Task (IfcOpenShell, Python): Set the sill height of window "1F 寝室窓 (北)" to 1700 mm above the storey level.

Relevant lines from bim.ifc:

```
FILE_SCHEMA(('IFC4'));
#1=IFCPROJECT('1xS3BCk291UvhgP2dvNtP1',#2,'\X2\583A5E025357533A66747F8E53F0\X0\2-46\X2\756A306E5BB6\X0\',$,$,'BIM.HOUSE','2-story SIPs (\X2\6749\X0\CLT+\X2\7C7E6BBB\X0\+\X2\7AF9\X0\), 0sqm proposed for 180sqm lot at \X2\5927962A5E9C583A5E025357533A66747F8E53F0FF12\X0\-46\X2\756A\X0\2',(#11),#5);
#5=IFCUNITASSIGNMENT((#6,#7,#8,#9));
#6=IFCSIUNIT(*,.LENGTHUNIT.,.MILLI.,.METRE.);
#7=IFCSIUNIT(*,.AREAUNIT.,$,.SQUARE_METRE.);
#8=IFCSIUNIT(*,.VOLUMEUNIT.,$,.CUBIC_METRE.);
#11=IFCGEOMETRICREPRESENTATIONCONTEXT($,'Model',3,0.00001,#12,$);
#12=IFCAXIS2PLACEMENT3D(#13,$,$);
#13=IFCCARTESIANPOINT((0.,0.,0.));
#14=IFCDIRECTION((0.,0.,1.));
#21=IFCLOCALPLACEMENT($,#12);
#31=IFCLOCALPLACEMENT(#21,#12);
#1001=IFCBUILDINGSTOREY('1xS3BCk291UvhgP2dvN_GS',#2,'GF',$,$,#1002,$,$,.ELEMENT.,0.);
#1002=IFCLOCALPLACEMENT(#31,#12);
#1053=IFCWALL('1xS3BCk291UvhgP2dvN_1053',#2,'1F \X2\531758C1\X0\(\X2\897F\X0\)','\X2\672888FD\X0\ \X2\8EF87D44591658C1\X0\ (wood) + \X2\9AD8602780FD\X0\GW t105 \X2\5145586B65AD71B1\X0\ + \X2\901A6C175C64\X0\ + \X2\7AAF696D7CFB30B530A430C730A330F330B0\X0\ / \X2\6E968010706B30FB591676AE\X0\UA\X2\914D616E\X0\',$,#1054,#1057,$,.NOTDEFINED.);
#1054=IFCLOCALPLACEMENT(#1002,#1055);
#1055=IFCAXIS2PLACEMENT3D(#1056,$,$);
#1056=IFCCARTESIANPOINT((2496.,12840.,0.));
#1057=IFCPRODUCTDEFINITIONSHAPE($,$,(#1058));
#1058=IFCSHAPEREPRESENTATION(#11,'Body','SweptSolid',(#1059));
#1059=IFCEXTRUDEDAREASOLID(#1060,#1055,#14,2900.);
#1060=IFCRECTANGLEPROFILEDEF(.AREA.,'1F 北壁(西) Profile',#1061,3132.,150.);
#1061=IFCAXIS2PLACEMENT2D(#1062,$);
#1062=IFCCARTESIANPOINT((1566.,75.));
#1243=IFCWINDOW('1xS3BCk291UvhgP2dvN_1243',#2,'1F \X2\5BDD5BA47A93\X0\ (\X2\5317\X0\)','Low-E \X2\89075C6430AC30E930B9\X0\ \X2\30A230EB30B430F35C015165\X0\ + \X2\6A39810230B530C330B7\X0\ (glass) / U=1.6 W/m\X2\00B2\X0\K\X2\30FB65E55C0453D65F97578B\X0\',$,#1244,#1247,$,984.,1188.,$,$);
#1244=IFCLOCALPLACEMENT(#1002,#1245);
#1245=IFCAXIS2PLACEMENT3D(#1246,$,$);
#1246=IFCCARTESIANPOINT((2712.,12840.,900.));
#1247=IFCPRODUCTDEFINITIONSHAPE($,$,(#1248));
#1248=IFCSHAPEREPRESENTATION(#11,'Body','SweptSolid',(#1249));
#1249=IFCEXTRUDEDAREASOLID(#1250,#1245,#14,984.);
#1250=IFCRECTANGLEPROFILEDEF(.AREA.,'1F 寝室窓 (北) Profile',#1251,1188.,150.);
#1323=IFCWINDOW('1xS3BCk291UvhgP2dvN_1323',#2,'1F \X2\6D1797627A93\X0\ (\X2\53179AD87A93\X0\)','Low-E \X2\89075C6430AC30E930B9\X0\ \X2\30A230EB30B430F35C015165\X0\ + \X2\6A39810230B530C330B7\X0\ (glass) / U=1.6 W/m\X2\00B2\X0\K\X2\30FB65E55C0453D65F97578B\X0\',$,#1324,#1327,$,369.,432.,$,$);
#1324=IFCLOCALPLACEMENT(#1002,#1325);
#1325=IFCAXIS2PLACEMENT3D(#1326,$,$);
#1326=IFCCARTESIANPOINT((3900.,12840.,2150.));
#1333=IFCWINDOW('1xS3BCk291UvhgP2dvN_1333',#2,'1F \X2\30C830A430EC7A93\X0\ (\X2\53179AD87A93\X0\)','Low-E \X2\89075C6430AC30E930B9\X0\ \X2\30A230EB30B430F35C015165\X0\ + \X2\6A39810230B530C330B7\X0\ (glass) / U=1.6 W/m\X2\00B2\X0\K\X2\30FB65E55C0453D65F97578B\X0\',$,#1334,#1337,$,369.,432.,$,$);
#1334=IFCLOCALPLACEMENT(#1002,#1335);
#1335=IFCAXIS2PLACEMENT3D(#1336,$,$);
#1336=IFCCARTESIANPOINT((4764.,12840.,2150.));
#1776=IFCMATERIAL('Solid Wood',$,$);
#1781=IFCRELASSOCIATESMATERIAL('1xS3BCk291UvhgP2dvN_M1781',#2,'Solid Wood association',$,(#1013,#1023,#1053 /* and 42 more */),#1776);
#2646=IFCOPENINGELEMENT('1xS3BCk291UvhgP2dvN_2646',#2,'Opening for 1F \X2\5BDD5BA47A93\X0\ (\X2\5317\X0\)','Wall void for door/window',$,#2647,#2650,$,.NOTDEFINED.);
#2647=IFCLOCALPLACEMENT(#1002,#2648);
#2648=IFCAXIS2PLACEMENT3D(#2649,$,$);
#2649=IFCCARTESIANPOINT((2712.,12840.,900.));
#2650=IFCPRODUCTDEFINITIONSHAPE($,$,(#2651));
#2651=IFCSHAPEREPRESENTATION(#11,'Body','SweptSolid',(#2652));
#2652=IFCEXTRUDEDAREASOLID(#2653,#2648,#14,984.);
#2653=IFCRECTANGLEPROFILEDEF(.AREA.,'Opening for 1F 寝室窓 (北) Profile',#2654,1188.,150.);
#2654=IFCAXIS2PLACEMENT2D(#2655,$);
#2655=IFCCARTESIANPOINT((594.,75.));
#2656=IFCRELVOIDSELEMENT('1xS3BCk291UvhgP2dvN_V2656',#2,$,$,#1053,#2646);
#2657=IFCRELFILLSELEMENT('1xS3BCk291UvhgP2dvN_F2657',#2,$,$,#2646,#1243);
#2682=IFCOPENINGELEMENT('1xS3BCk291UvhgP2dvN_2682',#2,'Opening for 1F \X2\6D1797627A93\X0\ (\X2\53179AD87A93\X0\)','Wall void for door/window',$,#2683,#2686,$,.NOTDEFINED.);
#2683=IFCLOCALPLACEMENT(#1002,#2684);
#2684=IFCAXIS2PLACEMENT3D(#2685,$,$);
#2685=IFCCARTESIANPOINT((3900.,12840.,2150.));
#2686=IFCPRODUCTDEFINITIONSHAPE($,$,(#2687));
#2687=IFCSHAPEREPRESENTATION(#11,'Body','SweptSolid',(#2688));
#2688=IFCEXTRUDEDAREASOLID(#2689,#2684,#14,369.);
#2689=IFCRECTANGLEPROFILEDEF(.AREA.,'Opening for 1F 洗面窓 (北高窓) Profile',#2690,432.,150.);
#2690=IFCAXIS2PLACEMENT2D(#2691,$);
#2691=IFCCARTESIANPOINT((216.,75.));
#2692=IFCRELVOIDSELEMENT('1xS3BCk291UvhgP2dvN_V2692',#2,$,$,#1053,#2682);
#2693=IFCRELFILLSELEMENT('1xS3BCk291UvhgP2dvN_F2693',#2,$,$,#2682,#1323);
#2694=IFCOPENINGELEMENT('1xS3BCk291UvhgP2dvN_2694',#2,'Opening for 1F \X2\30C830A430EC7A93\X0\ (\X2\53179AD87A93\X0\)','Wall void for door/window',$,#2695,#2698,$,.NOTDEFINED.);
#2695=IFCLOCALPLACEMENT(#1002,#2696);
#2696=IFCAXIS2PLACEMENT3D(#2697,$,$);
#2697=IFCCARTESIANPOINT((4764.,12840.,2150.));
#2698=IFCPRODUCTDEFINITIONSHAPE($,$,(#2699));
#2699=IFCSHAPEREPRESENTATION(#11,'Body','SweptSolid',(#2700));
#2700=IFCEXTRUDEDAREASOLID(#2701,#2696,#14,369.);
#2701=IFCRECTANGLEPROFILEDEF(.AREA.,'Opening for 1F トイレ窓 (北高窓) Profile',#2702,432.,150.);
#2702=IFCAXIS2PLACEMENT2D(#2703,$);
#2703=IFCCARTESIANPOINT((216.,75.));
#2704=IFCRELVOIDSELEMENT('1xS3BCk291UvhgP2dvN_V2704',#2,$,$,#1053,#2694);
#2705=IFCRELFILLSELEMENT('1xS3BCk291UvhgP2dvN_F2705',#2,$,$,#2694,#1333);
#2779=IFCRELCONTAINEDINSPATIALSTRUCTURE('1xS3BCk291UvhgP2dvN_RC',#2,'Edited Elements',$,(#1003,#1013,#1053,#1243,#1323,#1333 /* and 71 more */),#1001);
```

```python
import numpy as np
import ifcopenshell
import ifcopenshell.api.geometry
import ifcopenshell.geom
import ifcopenshell.util.element
import ifcopenshell.util.placement
import ifcopenshell.util.shape
import ifcopenshell.util.unit

model = ifcopenshell.open("bim.ifc")
unit_scale = ifcopenshell.util.unit.calculate_unit_scale(model)

window = model.by_guid("1xS3BCk291UvhgP2dvN_1243")
opening = window.FillsVoids[0].RelatingOpeningElement
storey = ifcopenshell.util.element.get_container(window, ifc_class="IfcBuildingStorey")
level = ifcopenshell.util.placement.get_local_placement(storey.ObjectPlacement)[2, 3]

# The opening's origin need not be at the sill, so measure its lowest point.
shape = ifcopenshell.geom.create_shape(ifcopenshell.geom.settings(), opening)
bottom = ifcopenshell.util.shape.get_shape_bottom_elevation(shape, shape.geometry) / unit_scale
dz = level + 1.7 / unit_scale - bottom

shift = np.array([0.0, 0.0, dz])
# The window is not placed relative to its opening, so move both.
for product in (opening, window):
    matrix = ifcopenshell.util.placement.get_local_placement(product.ObjectPlacement)
    matrix[:3, 3] += shift
    ifcopenshell.api.geometry.edit_object_placement(model, product=product, matrix=matrix, is_si=False)

print(f"moved by {dz * unit_scale:+.3f} m")

model.write("bim_rev.ifc")
```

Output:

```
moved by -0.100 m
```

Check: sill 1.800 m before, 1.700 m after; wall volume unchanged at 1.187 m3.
